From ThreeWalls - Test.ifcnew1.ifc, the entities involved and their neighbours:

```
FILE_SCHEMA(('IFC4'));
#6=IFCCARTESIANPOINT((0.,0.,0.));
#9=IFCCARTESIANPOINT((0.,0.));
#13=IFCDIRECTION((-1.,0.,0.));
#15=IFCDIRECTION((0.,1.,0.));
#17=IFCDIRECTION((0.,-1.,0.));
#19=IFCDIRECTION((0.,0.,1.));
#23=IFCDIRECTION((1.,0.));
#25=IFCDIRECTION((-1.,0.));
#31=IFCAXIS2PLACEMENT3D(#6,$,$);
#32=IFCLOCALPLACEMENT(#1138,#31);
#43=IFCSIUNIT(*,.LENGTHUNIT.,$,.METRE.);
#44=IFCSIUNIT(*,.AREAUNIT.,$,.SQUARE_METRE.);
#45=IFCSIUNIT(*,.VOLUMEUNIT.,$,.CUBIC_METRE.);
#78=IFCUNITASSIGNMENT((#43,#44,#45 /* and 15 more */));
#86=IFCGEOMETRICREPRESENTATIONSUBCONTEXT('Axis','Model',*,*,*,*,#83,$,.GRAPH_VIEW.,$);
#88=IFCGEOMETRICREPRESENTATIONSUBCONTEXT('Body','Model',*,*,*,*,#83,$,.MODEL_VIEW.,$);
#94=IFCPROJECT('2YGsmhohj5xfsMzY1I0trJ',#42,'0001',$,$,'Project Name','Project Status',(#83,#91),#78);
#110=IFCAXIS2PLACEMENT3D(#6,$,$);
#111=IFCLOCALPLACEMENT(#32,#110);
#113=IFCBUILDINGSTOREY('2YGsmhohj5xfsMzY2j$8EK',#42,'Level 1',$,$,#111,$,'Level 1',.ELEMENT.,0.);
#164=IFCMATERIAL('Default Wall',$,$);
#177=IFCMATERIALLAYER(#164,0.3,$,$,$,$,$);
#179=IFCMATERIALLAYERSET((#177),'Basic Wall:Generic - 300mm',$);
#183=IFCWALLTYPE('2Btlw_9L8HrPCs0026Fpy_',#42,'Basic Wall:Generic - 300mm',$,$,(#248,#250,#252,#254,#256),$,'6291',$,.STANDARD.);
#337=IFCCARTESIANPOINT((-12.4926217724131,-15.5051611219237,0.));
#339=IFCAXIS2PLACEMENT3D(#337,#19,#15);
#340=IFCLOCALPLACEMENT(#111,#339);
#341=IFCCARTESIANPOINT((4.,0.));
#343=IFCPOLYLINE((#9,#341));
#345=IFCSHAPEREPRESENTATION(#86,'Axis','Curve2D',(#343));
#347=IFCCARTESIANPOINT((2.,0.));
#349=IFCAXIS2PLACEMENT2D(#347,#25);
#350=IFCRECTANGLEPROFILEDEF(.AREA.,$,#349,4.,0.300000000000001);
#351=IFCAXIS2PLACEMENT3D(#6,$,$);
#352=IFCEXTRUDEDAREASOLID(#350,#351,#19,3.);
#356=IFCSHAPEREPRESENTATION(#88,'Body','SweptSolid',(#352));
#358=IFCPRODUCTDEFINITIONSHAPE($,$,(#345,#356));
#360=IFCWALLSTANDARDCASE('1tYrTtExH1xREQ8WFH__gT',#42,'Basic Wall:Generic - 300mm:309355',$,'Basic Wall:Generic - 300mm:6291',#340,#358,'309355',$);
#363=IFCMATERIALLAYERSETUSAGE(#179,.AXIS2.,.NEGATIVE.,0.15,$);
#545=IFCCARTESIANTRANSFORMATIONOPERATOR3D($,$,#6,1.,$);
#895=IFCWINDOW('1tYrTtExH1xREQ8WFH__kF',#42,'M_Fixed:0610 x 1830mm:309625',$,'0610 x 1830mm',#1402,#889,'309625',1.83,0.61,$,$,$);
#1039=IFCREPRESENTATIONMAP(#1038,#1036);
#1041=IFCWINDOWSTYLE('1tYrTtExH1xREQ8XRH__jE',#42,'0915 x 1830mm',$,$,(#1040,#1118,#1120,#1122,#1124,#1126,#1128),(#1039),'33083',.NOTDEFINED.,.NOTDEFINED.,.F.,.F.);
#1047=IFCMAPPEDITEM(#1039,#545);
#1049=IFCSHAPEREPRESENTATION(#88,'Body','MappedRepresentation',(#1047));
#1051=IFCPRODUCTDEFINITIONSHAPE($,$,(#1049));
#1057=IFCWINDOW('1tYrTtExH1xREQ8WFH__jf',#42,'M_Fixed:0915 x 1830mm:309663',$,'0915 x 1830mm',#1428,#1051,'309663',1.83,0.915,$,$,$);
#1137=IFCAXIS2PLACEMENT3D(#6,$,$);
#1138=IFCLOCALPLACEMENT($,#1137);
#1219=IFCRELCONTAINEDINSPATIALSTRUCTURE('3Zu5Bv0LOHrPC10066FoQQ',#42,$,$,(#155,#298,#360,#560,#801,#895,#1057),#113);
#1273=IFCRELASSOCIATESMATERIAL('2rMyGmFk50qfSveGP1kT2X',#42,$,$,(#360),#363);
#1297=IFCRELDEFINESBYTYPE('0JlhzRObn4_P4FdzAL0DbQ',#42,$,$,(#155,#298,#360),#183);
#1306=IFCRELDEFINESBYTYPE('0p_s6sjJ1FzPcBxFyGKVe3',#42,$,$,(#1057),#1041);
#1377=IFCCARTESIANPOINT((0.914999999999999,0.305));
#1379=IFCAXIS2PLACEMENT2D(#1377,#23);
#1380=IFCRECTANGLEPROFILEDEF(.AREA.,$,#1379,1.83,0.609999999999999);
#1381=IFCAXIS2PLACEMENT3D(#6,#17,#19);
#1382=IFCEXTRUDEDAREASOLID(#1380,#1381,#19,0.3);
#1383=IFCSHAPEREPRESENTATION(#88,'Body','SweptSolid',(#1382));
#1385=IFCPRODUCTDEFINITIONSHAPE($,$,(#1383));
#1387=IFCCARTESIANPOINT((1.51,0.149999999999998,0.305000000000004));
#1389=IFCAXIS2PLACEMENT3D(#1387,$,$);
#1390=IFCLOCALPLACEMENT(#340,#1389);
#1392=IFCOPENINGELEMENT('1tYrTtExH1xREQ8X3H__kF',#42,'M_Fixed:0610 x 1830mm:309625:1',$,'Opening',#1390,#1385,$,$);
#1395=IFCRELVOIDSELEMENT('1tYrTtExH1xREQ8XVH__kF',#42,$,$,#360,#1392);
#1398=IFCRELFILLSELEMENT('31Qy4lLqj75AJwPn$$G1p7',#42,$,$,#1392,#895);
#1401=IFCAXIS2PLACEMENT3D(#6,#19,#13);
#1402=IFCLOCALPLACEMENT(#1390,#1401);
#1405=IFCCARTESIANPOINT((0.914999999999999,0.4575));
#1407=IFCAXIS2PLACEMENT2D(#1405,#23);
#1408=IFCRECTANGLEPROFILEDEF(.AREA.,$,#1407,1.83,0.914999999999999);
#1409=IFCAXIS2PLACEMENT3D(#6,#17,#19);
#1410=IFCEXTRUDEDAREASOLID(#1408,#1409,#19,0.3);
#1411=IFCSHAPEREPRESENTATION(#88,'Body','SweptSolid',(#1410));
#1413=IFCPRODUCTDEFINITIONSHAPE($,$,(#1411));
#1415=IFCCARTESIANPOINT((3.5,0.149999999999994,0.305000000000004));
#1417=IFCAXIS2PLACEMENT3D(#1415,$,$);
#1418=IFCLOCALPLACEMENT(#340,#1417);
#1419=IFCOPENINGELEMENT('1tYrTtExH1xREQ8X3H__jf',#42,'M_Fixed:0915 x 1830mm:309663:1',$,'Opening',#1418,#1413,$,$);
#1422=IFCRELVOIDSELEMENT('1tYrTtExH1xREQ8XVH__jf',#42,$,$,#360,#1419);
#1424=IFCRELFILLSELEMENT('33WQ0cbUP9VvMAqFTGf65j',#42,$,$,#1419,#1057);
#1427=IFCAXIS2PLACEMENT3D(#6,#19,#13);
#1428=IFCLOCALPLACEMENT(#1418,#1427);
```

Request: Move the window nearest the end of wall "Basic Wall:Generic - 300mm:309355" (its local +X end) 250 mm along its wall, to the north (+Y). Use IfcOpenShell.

```python
import ifcopenshell
import ifcopenshell.api.geometry
import ifcopenshell.util.placement
import ifcopenshell.util.unit

model = ifcopenshell.open("ThreeWalls - Test.ifcnew1.ifc")
unit_scale = ifcopenshell.util.unit.calculate_unit_scale(model)

window = model.by_guid("1tYrTtExH1xREQ8WFH__jf")
opening = window.FillsVoids[0].RelatingOpeningElement
wall = opening.VoidsElements[0].RelatingBuildingElement

wall_matrix = ifcopenshell.util.placement.get_local_placement(wall.ObjectPlacement)
shift = wall_matrix[:3, 0] * 0.25 / unit_scale
before = ifcopenshell.util.placement.get_local_placement(window.ObjectPlacement)[:3, 3].copy()

# The window is placed relative to its opening, so it follows when the opening moves.
matrix = ifcopenshell.util.placement.get_local_placement(opening.ObjectPlacement)
matrix[:3, 3] += shift
ifcopenshell.api.geometry.edit_object_placement(
    model, product=opening, matrix=matrix, is_si=False, should_transform_children=True
)

after = ifcopenshell.util.placement.get_local_placement(window.ObjectPlacement)[:3, 3]
print("window moved by", (after - before).round(3) + 0.0)

model.write("ThreeWalls - Test.ifcnew1-out.ifc")
```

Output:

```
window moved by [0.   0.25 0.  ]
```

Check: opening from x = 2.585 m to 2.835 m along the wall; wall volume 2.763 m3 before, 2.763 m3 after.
